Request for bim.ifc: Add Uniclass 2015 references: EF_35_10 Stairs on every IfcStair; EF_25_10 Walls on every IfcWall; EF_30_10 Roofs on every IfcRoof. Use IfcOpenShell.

First a look at what the model holds.

```python
import ifcopenshell

model = ifcopenshell.open("bim.ifc")
print(model.schema)
print("classifications:", [c.Name for c in model.by_type("IfcClassification")])
for ifc_class in ("IfcDoor", "IfcRoof", "IfcStair", "IfcWall", "IfcWindow"):
    print(ifc_class, len(model.by_type(ifc_class)))
```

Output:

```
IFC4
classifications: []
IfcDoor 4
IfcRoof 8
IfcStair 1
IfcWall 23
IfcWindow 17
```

```python
import ifcopenshell
import ifcopenshell.api.classification

model = ifcopenshell.open("bim.ifc")

system = ifcopenshell.api.classification.add_classification(model, classification="Uniclass 2015")

codes = {
    "IfcStair": ("EF_35_10", "Stairs"),
    "IfcWall": ("EF_25_10", "Walls"),
    "IfcRoof": ("EF_30_10", "Roofs"),
}
for ifc_class, (code, name) in codes.items():
    products = model.by_type(ifc_class)
    ifcopenshell.api.classification.add_reference(
        model, products=products, classification=system, identification=code, name=name
    )
    print(code, len(products))

model.write("bim_v2.ifc")
```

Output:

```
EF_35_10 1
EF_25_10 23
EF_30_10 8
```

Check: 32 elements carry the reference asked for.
